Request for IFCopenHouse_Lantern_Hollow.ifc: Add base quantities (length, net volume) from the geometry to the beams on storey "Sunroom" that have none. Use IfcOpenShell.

First a look at what the model holds.

```python
import ifcopenshell
import ifcopenshell.util.element
import ifcopenshell.util.unit

model = ifcopenshell.open("IFCopenHouse_Lantern_Hollow.ifc")
print(model.schema)
for unit_type in ("LENGTHUNIT", "AREAUNIT", "VOLUMEUNIT"):
    print(unit_type, ifcopenshell.util.unit.calculate_unit_scale(model, unit_type))
storey = next(s for s in model.by_type("IfcBuildingStorey") if s.Name == "Sunroom")
beams = [e for e in ifcopenshell.util.element.get_decomposition(storey) if e.is_a("IfcBeam")]
for e in sorted(beams, key=lambda e: e.id()):
    print(e.id(), e.is_a(), e.Name, list(ifcopenshell.util.element.get_psets(e, qtos_only=True)), sep=" | ")
```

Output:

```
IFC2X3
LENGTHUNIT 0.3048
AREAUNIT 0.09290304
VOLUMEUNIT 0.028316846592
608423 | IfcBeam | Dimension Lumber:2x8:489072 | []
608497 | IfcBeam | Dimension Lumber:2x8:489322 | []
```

```python
import ifcopenshell
import ifcopenshell.api.pset
import ifcopenshell.geom
import ifcopenshell.util.element
import ifcopenshell.util.shape
import ifcopenshell.util.unit

model = ifcopenshell.open("IFCopenHouse_Lantern_Hollow.ifc")
unit_scale = ifcopenshell.util.unit.calculate_unit_scale(model)
volume_scale = ifcopenshell.util.unit.calculate_unit_scale(model, "VOLUMEUNIT")
settings = ifcopenshell.geom.settings()

storey = next(s for s in model.by_type("IfcBuildingStorey") if s.Name == "Sunroom")
beams = [e for e in ifcopenshell.util.element.get_decomposition(storey) if e.is_a("IfcBeam")]

for e in sorted(beams, key=lambda e: e.id()):
    if ifcopenshell.util.element.get_psets(e, qtos_only=True, should_inherit=False):
        continue
    # Geometry comes back in metres, in the element's own axes.
    shape = ifcopenshell.geom.create_shape(settings, e)
    values = {
        "Length": ifcopenshell.util.shape.get_max_xyz(shape.geometry) / unit_scale,
        "NetVolume": ifcopenshell.util.shape.get_volume(shape.geometry) / volume_scale,
    }
    qto = ifcopenshell.api.pset.add_qto(model, product=e, name="BaseQuantities")
    ifcopenshell.api.pset.edit_qto(model, qto=qto, properties=values)
    print(e.id(), {k: round(v, 3) for k, v in values.items()})

model.write("IFCopenHouse_Lantern_Hollow_updated.ifc")
```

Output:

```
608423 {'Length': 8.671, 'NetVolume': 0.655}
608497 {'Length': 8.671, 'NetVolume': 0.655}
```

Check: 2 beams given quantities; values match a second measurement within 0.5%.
